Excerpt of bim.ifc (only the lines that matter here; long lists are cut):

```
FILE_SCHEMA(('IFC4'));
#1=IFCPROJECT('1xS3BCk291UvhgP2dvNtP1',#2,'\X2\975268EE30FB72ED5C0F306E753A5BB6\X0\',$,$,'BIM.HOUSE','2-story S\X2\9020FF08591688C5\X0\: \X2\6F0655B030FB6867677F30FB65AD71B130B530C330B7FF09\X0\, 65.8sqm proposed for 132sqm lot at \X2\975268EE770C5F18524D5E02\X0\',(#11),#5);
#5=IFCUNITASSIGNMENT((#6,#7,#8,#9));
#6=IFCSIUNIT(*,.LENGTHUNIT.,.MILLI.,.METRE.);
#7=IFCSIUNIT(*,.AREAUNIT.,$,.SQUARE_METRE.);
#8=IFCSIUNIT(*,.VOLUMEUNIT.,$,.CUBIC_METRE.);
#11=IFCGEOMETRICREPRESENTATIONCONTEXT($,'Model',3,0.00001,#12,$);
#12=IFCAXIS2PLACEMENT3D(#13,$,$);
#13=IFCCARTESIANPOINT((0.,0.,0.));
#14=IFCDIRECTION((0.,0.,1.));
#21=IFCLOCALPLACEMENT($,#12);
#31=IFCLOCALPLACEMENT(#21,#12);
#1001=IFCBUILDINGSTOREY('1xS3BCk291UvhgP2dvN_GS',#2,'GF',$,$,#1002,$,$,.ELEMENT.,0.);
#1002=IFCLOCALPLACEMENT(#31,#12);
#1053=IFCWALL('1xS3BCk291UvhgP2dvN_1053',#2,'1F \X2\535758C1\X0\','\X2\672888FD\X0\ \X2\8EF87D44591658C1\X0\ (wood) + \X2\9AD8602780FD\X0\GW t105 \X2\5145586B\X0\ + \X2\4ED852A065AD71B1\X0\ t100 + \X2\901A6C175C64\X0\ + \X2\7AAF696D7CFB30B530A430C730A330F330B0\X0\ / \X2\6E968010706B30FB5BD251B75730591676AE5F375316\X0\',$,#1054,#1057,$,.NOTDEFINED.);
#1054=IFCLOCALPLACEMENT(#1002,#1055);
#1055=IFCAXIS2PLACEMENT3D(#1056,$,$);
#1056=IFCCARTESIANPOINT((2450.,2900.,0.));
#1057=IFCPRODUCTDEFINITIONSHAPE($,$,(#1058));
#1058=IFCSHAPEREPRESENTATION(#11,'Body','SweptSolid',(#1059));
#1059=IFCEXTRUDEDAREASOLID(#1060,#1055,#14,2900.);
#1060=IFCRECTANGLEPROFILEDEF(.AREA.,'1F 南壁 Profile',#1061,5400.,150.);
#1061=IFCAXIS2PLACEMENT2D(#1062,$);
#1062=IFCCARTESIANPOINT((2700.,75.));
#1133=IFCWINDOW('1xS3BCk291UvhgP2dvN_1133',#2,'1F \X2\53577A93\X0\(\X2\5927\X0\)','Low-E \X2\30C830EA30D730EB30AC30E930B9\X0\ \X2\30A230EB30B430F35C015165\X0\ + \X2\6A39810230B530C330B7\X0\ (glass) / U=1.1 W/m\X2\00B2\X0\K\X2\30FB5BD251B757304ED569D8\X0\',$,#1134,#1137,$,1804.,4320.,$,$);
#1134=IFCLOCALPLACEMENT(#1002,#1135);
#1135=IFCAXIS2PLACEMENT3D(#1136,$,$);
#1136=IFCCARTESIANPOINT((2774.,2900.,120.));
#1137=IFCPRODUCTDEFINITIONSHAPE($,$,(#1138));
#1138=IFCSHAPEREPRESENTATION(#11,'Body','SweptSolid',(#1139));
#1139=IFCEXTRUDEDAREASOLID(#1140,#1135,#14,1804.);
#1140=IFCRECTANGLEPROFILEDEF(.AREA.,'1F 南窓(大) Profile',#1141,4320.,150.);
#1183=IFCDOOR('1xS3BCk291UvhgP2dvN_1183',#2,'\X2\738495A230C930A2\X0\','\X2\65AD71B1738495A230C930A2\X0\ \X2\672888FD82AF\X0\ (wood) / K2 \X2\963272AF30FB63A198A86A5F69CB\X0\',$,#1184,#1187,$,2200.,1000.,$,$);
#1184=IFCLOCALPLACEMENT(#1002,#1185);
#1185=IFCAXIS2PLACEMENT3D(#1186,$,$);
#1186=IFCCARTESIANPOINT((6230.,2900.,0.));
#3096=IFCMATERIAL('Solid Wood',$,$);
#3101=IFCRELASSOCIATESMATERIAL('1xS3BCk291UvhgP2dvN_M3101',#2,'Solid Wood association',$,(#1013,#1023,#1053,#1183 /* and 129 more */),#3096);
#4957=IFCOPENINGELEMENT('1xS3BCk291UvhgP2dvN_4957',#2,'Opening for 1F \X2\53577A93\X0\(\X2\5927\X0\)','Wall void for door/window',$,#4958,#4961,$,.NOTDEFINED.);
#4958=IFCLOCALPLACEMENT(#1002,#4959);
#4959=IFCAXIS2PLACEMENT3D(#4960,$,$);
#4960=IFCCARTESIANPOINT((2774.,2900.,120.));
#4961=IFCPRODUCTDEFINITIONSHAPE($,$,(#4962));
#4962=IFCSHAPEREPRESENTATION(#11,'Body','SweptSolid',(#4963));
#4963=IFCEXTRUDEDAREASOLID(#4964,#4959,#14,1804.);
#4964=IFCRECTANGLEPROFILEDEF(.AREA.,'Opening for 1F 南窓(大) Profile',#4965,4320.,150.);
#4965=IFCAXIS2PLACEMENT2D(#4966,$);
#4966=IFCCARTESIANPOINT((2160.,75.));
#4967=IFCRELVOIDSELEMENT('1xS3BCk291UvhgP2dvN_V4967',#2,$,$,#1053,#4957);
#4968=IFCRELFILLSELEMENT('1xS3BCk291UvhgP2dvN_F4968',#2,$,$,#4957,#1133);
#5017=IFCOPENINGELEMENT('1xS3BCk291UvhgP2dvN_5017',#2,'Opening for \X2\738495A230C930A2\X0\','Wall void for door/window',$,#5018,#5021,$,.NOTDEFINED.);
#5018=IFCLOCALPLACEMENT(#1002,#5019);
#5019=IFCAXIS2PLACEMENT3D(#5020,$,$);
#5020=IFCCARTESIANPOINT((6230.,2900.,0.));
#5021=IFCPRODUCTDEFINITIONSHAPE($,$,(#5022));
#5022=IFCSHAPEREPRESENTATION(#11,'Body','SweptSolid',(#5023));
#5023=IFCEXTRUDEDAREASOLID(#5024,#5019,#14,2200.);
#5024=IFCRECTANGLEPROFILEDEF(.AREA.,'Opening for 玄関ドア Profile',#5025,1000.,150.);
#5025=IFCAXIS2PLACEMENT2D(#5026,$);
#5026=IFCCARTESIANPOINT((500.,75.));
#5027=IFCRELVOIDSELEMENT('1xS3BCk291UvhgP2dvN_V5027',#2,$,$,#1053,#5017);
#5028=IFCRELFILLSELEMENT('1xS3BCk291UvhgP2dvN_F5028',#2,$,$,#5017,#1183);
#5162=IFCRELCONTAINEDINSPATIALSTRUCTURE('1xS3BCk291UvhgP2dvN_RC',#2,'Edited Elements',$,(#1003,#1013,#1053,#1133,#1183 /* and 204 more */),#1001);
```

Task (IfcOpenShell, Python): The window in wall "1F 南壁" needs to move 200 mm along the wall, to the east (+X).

```python
import ifcopenshell
import ifcopenshell.api.geometry
import ifcopenshell.util.placement

model = ifcopenshell.open("bim.ifc")

window = model.by_guid("1xS3BCk291UvhgP2dvN_1133")
opening = window.FillsVoids[0].RelatingOpeningElement
wall = opening.VoidsElements[0].RelatingBuildingElement

wall_matrix = ifcopenshell.util.placement.get_local_placement(wall.ObjectPlacement)
shift = wall_matrix[:3, 0] * 200.0
before = ifcopenshell.util.placement.get_local_placement(window.ObjectPlacement)[:3, 3].copy()

# The window is not placed relative to its opening, so move both.
for product in (opening, window):
    matrix = ifcopenshell.util.placement.get_local_placement(product.ObjectPlacement)
    matrix[:3, 3] += shift
    ifcopenshell.api.geometry.edit_object_placement(model, product=product, matrix=matrix, is_si=False)

after = ifcopenshell.util.placement.get_local_placement(window.ObjectPlacement)[:3, 3]
print("window moved by", (after - before).round(3) + 0.0)

model.write("bim_updated.ifc")
```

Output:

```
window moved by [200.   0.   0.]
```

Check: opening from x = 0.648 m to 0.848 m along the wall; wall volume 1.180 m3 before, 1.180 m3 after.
